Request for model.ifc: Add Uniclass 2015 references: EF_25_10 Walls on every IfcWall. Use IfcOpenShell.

First a look at what the model holds.

```python
import ifcopenshell

model = ifcopenshell.open("model.ifc")
print(model.schema)
print("classifications:", [c.Name for c in model.by_type("IfcClassification")])
for ifc_class in ("IfcDoor", "IfcRoof", "IfcStair", "IfcWall", "IfcWindow"):
    print(ifc_class, len(model.by_type(ifc_class)))
```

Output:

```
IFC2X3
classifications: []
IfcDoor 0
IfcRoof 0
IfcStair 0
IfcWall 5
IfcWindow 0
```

```python
import ifcopenshell
import ifcopenshell.api.classification

model = ifcopenshell.open("model.ifc")

# IFC2X3 requires Source and Edition and has no link from the project to the system.
system = model.create_entity("IfcClassification", Source="NBS", Edition="2015", Name="Uniclass 2015")

codes = {
    "IfcWall": ("EF_25_10", "Walls"),
}
for ifc_class, (code, name) in codes.items():
    products = model.by_type(ifc_class)
    ifcopenshell.api.classification.add_reference(
        model, products=products, classification=system, identification=code, name=name
    )
    print(code, len(products))

model.write("model_updated.ifc")
```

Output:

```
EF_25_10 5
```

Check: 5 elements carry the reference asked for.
